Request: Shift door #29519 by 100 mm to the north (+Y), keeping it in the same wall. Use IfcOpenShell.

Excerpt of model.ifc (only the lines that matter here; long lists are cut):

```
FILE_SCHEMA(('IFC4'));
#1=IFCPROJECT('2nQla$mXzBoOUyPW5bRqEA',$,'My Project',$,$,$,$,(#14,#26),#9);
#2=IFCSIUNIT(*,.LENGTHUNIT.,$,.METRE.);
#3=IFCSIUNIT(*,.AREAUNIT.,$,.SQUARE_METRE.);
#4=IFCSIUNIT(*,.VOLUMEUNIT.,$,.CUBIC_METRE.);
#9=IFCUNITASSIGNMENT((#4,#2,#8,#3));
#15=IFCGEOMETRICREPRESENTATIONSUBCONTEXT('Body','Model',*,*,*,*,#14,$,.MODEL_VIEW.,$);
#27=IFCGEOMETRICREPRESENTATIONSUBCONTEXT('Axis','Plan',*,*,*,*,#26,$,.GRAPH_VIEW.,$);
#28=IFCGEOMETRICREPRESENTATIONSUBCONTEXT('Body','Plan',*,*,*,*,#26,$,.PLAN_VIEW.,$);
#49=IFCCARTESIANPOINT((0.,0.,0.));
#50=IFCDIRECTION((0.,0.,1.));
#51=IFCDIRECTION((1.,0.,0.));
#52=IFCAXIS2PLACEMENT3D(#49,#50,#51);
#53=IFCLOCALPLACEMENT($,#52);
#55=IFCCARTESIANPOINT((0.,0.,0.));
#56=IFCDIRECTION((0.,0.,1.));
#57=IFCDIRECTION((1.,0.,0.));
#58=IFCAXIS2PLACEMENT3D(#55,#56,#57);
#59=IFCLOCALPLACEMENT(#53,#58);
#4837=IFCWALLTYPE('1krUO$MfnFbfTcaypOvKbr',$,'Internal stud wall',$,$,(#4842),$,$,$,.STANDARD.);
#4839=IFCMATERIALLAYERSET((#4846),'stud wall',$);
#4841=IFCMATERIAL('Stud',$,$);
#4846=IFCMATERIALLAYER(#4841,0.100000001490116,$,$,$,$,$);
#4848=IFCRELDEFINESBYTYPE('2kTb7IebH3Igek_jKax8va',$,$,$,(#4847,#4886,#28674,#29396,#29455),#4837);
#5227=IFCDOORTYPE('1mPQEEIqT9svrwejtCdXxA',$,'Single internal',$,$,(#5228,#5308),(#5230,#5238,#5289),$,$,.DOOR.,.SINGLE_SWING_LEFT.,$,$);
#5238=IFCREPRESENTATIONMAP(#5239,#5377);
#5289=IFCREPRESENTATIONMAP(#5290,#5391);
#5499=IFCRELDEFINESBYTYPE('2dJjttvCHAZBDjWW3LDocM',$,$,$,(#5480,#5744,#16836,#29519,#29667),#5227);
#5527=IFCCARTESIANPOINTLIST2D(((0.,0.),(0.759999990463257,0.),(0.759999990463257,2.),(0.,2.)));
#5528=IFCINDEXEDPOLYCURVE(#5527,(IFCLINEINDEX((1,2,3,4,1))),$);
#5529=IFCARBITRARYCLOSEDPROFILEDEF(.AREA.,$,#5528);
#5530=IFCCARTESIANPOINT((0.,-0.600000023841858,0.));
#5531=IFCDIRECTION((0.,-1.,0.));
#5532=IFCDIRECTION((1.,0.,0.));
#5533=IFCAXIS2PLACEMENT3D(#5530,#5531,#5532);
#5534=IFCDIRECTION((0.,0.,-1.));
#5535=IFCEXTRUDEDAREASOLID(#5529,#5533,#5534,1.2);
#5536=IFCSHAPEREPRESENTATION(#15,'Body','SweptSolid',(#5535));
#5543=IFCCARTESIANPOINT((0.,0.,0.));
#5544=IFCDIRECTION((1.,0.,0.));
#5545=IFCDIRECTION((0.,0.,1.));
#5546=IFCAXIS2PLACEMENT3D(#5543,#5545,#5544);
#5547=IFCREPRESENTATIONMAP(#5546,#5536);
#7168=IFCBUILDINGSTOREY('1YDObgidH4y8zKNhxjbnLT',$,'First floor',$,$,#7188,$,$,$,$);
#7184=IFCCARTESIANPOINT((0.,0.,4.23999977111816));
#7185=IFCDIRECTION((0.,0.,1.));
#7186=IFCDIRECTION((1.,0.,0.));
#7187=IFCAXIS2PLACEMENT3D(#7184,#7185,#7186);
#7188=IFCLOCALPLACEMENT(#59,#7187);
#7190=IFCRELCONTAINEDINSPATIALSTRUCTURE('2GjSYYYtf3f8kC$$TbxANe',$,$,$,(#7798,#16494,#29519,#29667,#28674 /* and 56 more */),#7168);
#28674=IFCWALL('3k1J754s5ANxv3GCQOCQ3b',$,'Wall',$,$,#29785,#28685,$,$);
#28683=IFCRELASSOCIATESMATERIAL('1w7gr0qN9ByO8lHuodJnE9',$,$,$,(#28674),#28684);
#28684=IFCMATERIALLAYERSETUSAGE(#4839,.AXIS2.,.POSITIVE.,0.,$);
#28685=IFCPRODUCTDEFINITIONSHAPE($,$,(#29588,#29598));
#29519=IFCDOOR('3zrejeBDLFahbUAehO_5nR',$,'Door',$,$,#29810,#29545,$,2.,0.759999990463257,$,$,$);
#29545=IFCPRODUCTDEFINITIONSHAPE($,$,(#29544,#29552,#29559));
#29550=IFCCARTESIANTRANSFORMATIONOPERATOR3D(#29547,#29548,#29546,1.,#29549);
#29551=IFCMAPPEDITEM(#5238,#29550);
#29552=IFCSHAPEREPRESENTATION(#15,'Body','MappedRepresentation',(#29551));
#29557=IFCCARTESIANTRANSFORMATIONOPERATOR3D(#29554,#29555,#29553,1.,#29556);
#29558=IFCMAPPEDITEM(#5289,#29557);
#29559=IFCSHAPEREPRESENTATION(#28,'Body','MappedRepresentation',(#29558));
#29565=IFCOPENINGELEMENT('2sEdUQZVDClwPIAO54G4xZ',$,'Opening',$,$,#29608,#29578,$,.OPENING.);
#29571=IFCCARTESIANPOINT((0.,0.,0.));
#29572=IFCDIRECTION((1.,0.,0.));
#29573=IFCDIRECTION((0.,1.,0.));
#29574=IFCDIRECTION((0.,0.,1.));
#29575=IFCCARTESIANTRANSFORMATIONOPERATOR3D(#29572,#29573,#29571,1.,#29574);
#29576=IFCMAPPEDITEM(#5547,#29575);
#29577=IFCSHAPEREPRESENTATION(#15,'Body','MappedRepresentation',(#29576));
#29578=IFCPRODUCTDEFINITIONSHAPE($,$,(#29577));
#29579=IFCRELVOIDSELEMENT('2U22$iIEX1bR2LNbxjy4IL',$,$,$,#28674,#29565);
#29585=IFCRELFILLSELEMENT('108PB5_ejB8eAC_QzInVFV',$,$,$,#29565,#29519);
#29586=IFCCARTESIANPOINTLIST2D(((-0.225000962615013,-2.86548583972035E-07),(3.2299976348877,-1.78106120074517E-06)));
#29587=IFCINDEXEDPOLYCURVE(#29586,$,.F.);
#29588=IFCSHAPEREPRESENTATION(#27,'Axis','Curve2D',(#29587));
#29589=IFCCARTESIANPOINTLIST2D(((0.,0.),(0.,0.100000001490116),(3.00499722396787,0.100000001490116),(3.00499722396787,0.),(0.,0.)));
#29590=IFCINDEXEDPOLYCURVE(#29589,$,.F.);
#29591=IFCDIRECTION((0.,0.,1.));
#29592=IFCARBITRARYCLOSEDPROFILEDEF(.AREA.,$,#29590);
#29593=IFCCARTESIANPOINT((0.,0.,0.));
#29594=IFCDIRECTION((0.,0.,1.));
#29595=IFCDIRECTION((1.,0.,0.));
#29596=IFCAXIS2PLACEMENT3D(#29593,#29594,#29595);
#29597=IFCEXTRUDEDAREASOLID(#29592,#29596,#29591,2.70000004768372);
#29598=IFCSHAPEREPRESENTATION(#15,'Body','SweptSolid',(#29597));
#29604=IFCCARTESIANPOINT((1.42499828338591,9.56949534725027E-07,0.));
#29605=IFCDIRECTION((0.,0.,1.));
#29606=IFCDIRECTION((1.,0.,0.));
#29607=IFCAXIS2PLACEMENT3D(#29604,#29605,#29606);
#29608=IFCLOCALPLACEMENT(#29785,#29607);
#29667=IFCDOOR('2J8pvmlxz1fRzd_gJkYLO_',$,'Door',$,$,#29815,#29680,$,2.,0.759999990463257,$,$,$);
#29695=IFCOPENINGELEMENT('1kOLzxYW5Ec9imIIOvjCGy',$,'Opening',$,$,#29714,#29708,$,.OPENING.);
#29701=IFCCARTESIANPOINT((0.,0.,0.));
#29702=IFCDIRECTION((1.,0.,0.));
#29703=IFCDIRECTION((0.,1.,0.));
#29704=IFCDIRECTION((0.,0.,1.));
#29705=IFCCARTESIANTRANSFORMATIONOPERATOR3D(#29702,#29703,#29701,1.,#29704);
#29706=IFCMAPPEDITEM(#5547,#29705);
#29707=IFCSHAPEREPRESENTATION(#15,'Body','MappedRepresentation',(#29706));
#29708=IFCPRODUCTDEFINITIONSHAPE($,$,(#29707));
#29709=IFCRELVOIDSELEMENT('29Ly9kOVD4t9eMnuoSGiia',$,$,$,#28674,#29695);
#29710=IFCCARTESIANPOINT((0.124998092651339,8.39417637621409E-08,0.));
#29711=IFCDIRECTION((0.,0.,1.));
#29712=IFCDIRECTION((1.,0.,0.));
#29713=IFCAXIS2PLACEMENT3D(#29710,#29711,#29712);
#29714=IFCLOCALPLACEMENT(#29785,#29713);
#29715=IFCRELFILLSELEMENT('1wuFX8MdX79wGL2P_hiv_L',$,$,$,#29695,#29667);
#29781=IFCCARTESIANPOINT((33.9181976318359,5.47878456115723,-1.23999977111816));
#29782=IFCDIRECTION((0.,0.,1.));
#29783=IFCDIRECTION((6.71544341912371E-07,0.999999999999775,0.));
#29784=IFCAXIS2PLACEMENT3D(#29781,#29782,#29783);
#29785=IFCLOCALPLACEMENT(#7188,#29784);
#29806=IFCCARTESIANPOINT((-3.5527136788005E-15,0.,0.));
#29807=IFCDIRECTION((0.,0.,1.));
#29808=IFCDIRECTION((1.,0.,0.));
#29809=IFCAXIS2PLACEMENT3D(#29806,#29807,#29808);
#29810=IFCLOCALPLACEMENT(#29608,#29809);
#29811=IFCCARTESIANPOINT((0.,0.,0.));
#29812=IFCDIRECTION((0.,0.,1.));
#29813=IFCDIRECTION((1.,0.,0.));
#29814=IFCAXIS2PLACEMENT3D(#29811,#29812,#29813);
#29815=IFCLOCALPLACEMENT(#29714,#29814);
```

```python
import ifcopenshell
import ifcopenshell.api.geometry
import ifcopenshell.util.placement
import ifcopenshell.util.unit

model = ifcopenshell.open("model.ifc")
unit_scale = ifcopenshell.util.unit.calculate_unit_scale(model)

door = model.by_guid("3zrejeBDLFahbUAehO_5nR")
opening = door.FillsVoids[0].RelatingOpeningElement
wall = opening.VoidsElements[0].RelatingBuildingElement

wall_matrix = ifcopenshell.util.placement.get_local_placement(wall.ObjectPlacement)
shift = wall_matrix[:3, 0] * 0.1 / unit_scale
before = ifcopenshell.util.placement.get_local_placement(door.ObjectPlacement)[:3, 3].copy()

# The door is placed relative to its opening, so it follows when the opening moves.
matrix = ifcopenshell.util.placement.get_local_placement(opening.ObjectPlacement)
matrix[:3, 3] += shift
ifcopenshell.api.geometry.edit_object_placement(
    model, product=opening, matrix=matrix, is_si=False, should_transform_children=True
)

after = ifcopenshell.util.placement.get_local_placement(door.ObjectPlacement)[:3, 3]
print("door moved by", (after - before).round(3) + 0.0)

model.write("model_edited.ifc")
```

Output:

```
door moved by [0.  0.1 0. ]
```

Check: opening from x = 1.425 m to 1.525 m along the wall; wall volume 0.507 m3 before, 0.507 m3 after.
